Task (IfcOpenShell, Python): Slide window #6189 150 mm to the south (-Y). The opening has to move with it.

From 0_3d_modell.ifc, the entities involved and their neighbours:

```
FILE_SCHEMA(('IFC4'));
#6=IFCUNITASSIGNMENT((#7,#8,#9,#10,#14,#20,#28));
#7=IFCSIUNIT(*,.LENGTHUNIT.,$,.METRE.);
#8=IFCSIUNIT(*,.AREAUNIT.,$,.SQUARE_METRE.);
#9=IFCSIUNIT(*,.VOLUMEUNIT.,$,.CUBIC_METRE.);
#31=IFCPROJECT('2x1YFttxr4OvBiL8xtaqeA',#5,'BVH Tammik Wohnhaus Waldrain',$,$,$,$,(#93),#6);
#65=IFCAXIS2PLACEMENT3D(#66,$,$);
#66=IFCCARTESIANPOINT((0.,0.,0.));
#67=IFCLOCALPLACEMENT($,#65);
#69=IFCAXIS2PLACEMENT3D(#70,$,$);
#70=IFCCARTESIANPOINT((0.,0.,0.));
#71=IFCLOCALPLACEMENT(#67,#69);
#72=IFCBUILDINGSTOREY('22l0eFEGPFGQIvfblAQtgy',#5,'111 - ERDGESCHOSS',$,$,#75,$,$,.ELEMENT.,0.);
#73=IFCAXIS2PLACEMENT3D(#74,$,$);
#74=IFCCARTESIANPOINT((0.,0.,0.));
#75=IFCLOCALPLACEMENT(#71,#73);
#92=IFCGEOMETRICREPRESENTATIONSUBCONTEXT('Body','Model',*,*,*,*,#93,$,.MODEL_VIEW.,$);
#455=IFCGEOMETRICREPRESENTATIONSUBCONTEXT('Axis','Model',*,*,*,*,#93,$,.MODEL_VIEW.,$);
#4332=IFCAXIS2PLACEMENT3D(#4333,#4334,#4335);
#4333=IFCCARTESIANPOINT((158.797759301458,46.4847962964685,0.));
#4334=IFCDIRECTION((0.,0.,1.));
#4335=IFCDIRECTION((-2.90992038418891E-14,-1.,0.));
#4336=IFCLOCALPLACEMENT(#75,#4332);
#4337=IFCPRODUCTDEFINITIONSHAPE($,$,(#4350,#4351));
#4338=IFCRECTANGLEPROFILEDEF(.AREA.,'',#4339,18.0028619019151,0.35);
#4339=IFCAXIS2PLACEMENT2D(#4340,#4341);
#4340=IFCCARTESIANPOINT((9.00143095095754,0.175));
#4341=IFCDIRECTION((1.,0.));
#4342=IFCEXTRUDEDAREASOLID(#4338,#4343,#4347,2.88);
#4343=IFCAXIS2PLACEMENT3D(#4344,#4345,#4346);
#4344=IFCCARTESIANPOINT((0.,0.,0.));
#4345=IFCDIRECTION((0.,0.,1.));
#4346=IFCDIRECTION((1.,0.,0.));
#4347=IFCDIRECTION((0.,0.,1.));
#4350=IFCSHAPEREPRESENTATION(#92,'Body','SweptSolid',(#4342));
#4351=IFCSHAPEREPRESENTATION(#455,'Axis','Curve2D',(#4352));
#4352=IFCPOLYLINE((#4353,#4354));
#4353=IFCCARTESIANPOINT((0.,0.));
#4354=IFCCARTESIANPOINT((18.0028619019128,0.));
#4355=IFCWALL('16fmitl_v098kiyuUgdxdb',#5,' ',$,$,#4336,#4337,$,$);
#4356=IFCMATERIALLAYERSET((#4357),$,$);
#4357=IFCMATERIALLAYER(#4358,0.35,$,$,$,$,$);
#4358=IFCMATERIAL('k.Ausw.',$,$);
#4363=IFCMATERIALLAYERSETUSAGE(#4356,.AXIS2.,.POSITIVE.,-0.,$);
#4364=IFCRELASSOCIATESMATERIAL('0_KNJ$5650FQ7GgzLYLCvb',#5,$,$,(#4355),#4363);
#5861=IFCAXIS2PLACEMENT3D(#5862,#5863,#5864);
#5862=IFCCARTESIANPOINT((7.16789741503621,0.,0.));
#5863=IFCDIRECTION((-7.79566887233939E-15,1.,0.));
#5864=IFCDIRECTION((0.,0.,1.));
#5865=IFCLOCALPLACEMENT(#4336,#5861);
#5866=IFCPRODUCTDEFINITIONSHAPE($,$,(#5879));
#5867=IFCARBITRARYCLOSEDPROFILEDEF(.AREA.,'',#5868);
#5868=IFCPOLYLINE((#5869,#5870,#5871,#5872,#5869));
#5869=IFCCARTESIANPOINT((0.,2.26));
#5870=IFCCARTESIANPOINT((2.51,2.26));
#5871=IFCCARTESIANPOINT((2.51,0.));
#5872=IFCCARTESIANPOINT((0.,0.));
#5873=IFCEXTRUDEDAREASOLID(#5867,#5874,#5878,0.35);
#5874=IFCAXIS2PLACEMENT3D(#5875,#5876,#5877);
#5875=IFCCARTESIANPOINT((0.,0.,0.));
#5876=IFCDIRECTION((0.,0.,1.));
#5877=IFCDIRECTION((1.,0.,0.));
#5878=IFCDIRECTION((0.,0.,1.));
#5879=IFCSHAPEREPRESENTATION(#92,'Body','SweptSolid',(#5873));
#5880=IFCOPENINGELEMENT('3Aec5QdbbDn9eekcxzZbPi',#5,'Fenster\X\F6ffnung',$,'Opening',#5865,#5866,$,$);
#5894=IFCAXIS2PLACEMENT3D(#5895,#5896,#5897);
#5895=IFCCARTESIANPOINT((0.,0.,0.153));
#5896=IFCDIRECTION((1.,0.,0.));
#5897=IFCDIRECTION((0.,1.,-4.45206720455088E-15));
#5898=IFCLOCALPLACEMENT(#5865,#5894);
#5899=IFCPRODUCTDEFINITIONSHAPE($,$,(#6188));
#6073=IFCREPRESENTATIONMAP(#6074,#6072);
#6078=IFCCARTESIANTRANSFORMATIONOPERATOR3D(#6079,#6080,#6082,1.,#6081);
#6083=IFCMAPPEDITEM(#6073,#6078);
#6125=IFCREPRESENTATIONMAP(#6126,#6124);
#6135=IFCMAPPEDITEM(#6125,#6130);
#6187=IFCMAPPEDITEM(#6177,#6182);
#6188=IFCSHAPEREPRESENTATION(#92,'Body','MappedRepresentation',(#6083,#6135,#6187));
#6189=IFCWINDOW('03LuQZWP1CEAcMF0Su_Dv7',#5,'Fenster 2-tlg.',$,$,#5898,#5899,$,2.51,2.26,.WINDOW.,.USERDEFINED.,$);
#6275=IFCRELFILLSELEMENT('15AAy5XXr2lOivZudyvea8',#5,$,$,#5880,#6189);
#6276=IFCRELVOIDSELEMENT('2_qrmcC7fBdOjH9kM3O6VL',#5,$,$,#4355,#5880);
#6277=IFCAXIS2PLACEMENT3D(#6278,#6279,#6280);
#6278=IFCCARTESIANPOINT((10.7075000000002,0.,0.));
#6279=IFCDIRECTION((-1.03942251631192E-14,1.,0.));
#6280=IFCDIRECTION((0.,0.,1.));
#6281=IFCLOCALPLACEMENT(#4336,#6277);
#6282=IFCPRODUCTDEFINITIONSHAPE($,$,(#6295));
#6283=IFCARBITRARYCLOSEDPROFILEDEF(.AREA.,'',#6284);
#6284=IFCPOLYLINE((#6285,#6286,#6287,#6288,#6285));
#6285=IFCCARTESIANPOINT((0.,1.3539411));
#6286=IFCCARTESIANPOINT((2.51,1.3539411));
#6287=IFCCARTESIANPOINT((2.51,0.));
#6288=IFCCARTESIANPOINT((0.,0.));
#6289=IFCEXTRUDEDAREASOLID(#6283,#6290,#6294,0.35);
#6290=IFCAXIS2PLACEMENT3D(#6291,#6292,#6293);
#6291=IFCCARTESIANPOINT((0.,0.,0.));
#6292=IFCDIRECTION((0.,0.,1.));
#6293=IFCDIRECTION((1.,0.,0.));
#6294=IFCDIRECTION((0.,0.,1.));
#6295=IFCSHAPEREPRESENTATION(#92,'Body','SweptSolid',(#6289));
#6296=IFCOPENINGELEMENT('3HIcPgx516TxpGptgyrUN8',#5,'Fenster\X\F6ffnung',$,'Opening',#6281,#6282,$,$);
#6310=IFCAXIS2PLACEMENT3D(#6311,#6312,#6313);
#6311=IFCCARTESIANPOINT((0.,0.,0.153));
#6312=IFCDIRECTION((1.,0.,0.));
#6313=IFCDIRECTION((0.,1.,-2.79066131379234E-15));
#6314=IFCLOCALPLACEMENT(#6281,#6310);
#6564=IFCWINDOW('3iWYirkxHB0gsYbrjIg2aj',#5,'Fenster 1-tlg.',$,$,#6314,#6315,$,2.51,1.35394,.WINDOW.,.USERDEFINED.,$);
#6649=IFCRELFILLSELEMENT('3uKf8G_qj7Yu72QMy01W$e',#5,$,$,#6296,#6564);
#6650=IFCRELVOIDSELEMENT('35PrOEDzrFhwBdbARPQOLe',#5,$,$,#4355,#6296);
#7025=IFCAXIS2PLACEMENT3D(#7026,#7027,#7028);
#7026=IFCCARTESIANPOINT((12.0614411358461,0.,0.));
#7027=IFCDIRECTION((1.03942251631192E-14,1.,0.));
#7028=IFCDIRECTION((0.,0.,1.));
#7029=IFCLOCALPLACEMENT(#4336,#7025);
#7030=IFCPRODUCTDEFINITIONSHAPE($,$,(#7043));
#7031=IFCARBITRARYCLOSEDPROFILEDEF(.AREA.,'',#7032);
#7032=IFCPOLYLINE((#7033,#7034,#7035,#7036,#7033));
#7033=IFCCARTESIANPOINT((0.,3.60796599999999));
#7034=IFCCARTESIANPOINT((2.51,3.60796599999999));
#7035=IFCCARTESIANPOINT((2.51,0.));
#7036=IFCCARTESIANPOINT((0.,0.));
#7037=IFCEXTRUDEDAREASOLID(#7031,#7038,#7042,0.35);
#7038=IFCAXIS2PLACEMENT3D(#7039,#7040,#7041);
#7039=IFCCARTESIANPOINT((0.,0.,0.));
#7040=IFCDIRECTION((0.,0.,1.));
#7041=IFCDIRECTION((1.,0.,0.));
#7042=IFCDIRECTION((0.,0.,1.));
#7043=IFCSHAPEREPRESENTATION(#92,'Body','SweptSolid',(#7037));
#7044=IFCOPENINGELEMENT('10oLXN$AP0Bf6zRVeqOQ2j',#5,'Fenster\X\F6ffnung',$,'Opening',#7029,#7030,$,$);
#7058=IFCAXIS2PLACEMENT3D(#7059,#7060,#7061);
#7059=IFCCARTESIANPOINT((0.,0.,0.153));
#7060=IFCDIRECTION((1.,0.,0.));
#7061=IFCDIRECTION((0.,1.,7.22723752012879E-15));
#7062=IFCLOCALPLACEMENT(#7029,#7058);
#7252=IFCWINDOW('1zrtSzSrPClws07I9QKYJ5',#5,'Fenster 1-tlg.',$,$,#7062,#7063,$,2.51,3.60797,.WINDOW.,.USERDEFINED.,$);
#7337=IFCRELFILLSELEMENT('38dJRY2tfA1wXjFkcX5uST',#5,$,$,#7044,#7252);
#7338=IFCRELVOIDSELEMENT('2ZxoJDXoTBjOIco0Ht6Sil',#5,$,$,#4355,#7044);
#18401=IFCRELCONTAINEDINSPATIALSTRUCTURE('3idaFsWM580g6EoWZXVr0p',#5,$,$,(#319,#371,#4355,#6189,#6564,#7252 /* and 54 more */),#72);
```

```python
import ifcopenshell
import ifcopenshell.api.geometry
import ifcopenshell.util.placement
import ifcopenshell.util.unit

model = ifcopenshell.open("0_3d_modell.ifc")
unit_scale = ifcopenshell.util.unit.calculate_unit_scale(model)

window = model.by_id(6189)
opening = window.FillsVoids[0].RelatingOpeningElement
wall = opening.VoidsElements[0].RelatingBuildingElement

wall_matrix = ifcopenshell.util.placement.get_local_placement(wall.ObjectPlacement)
shift = wall_matrix[:3, 0] * 0.15 / unit_scale
before = ifcopenshell.util.placement.get_local_placement(window.ObjectPlacement)[:3, 3].copy()

# The window is placed relative to its opening, so it follows when the opening moves.
matrix = ifcopenshell.util.placement.get_local_placement(opening.ObjectPlacement)
matrix[:3, 3] += shift
ifcopenshell.api.geometry.edit_object_placement(
    model, product=opening, matrix=matrix, is_si=False, should_transform_children=True
)

after = ifcopenshell.util.placement.get_local_placement(window.ObjectPlacement)[:3, 3]
print("window moved by", (after - before).round(3) + 0.0)

model.write("0_3d_modell-out.ifc")
```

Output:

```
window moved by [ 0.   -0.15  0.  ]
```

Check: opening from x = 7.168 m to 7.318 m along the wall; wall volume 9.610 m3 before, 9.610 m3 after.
